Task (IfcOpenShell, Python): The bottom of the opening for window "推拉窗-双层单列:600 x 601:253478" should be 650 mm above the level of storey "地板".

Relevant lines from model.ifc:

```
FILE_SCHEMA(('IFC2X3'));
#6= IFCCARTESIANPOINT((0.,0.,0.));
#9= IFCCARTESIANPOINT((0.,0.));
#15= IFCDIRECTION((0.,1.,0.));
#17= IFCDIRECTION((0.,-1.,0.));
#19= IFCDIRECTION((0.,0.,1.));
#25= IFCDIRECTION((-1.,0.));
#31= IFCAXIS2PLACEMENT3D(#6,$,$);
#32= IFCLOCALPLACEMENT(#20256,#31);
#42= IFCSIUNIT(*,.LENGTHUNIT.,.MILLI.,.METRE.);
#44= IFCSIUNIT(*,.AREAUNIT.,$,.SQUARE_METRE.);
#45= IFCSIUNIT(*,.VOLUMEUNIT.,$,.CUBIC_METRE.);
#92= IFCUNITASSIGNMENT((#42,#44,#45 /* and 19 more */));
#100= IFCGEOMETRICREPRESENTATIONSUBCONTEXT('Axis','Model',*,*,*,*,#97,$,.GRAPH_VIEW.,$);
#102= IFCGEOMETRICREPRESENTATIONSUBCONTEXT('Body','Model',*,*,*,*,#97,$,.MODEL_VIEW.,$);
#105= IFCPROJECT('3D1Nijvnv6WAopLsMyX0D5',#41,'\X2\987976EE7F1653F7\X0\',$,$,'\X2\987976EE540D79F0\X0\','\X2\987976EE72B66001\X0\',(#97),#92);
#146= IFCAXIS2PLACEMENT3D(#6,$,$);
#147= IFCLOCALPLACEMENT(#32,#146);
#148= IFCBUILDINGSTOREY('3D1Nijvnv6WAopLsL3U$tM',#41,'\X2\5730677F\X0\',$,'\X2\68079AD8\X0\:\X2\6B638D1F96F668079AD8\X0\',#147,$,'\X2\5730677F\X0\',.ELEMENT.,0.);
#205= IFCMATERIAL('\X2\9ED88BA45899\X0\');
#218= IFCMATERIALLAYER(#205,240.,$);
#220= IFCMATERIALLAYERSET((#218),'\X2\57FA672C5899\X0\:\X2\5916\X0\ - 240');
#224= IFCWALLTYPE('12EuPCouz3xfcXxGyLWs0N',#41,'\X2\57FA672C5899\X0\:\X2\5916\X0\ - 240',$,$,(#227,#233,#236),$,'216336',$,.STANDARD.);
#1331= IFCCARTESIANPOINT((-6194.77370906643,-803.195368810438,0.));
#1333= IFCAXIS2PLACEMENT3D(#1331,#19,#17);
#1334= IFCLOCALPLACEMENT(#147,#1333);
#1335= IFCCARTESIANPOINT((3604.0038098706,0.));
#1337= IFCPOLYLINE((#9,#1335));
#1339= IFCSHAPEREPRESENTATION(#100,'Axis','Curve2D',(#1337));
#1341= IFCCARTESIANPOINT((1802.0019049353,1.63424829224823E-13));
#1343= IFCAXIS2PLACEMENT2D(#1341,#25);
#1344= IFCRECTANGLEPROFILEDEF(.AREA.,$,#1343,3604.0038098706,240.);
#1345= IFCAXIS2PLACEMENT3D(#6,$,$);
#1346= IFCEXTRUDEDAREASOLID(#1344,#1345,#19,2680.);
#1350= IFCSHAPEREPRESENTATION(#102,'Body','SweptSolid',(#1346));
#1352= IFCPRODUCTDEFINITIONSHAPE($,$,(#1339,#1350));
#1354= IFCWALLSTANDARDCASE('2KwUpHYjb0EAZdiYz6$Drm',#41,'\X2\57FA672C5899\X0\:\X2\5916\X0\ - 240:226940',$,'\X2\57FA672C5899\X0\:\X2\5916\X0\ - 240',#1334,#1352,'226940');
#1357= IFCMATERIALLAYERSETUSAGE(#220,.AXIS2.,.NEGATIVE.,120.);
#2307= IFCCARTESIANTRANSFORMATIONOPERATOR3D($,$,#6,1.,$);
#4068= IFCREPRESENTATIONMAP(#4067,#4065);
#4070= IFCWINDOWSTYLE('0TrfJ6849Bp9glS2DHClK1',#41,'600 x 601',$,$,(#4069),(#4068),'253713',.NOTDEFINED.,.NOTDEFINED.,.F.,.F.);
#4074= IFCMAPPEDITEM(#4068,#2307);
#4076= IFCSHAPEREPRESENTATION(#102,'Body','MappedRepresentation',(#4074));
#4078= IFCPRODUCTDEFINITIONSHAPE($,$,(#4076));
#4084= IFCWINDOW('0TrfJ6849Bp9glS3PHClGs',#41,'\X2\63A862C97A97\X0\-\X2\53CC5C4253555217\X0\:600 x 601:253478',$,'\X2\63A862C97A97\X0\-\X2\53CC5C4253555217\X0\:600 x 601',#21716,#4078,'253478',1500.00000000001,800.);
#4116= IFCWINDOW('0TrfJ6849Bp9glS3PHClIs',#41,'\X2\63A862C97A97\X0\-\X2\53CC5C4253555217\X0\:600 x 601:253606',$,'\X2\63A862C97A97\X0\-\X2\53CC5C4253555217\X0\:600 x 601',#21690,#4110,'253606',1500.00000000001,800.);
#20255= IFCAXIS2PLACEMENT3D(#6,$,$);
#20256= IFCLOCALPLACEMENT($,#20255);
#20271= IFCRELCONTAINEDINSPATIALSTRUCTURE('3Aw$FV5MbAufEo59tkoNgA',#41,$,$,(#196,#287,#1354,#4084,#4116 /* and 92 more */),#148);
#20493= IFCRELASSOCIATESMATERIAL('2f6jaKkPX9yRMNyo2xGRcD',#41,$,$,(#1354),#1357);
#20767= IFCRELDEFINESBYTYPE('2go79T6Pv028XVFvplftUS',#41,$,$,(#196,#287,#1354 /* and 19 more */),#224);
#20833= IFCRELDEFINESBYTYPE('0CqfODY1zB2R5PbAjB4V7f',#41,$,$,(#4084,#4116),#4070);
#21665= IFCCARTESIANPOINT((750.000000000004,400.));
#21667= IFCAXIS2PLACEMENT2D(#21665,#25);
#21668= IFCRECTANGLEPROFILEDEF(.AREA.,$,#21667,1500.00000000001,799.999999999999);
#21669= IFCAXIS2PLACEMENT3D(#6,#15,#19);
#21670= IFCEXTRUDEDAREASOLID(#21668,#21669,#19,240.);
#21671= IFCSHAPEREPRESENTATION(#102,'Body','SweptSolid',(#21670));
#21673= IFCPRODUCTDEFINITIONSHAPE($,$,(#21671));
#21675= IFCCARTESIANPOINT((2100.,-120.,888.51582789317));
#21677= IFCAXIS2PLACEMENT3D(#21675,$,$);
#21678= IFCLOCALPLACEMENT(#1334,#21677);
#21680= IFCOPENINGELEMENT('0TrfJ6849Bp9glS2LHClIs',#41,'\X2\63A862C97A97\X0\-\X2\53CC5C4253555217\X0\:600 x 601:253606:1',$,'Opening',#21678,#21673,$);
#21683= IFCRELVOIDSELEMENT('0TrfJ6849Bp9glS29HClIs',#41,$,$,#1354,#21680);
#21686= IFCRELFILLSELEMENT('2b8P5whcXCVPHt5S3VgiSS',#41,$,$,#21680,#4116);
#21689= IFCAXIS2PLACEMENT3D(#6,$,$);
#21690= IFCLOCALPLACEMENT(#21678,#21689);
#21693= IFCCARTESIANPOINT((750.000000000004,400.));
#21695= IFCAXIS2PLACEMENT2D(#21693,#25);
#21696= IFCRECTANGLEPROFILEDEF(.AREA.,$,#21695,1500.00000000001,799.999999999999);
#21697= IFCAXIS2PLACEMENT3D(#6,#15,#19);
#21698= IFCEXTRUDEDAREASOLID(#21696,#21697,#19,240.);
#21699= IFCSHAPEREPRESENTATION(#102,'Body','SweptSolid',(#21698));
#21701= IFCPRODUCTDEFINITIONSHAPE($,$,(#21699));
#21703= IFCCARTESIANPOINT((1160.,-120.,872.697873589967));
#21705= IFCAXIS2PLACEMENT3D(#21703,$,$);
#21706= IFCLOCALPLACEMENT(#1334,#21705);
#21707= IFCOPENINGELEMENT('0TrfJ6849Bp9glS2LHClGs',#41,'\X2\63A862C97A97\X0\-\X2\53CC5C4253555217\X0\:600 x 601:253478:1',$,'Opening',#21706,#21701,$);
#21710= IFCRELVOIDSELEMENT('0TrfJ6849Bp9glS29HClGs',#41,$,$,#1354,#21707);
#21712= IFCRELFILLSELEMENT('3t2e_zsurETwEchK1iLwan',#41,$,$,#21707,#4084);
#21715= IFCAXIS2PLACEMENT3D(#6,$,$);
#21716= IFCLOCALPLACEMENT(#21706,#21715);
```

```python
import numpy as np
import ifcopenshell
import ifcopenshell.api.geometry
import ifcopenshell.geom
import ifcopenshell.util.element
import ifcopenshell.util.placement
import ifcopenshell.util.shape
import ifcopenshell.util.unit

model = ifcopenshell.open("model.ifc")
unit_scale = ifcopenshell.util.unit.calculate_unit_scale(model)

window = model.by_id(4084)
opening = window.FillsVoids[0].RelatingOpeningElement
storey = ifcopenshell.util.element.get_container(window, ifc_class="IfcBuildingStorey")
level = ifcopenshell.util.placement.get_local_placement(storey.ObjectPlacement)[2, 3]

# The opening's origin need not be at the sill, so measure its lowest point.
shape = ifcopenshell.geom.create_shape(ifcopenshell.geom.settings(), opening)
bottom = ifcopenshell.util.shape.get_shape_bottom_elevation(shape, shape.geometry) / unit_scale
dz = level + 650.0 - bottom

shift = np.array([0.0, 0.0, dz])
# The window is placed relative to its opening, so it follows when the opening moves.
matrix = ifcopenshell.util.placement.get_local_placement(opening.ObjectPlacement)
matrix[:3, 3] += shift
ifcopenshell.api.geometry.edit_object_placement(
    model, product=opening, matrix=matrix, is_si=False, should_transform_children=True
)

print(f"moved by {dz * unit_scale:+.3f} m")

model.write("model_v2.ifc")
```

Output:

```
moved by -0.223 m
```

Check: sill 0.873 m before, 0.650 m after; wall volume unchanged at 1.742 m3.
